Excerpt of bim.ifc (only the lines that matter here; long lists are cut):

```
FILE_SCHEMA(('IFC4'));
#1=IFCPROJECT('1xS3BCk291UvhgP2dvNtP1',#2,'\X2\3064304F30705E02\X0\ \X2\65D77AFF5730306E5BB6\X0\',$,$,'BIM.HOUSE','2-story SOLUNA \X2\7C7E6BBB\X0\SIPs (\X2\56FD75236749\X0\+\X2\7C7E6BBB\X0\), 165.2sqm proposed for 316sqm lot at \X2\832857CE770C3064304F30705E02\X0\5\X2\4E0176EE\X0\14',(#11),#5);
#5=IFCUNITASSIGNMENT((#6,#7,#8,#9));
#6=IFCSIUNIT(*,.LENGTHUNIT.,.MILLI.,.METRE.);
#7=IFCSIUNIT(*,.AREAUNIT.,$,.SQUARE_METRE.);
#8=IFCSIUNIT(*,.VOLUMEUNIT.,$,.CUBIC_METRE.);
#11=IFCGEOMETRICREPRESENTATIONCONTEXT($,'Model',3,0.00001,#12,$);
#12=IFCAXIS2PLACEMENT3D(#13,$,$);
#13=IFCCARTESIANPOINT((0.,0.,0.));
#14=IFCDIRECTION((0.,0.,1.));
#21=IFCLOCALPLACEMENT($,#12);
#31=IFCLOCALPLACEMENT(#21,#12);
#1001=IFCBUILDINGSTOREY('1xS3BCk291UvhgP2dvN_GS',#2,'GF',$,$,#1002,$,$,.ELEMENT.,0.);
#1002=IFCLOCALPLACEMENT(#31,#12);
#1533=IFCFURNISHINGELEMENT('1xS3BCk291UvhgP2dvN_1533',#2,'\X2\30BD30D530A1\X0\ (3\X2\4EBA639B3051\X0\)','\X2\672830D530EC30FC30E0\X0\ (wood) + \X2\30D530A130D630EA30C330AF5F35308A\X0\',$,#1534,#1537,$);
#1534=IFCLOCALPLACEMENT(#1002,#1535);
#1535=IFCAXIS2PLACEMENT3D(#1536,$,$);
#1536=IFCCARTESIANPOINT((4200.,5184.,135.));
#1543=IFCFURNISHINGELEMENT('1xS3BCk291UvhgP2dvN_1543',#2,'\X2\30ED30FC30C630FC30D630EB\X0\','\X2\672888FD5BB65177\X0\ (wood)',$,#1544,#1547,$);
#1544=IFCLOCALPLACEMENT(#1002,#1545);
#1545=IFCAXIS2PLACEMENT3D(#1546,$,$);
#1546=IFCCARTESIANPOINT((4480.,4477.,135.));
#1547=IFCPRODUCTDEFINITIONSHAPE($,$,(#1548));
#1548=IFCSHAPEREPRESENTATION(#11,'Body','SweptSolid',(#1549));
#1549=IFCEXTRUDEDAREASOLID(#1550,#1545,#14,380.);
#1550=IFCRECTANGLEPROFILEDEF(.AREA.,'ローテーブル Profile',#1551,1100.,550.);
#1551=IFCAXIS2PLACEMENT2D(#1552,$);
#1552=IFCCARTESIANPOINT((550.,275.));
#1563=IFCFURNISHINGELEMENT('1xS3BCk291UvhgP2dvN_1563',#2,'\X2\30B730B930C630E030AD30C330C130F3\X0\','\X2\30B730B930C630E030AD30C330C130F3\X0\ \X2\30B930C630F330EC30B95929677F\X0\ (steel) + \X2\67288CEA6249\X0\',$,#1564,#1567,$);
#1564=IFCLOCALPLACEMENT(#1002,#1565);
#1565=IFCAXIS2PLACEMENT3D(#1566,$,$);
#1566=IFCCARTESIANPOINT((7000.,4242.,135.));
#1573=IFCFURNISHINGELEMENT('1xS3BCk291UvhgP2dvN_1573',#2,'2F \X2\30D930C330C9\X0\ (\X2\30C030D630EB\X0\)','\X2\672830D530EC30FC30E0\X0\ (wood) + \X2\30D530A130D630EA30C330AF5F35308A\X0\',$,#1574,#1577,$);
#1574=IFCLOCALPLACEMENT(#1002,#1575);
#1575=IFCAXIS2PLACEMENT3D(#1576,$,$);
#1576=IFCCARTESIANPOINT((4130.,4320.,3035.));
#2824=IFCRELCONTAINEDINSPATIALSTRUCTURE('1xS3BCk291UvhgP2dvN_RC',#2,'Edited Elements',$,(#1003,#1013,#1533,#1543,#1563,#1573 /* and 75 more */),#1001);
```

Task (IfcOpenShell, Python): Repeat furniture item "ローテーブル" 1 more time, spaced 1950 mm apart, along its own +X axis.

```python
import ifcopenshell
import ifcopenshell.api.geometry
import ifcopenshell.api.root
import ifcopenshell.util.element
import ifcopenshell.util.placement

model = ifcopenshell.open("bim.ifc")


def reuse_history(source, copy):
    """copy_class also copies each property set's owner history, people and application; keep the originals."""
    for rel in copy.IsDefinedBy:
        if rel.is_a("IfcRelDefinesByProperties") and (history := rel.RelatingPropertyDefinition.OwnerHistory):
            rel.RelatingPropertyDefinition.OwnerHistory = source.OwnerHistory
            ifcopenshell.util.element.remove_deep2(model, history)


source = model.by_id(1543)
base = ifcopenshell.util.placement.get_local_placement(source.ObjectPlacement)
step = base[:3, 0] * 1950.0

for i in range(1, 2):
    copy = ifcopenshell.api.root.copy_class(model, product=source)
    copy.Representation = ifcopenshell.util.element.copy_deep(
        model, source.Representation, exclude=["IfcGeometricRepresentationContext", "IfcRepresentationMap"]
    )
    reuse_history(source, copy)
    matrix = base.copy()
    matrix[:3, 3] += i * step
    print("added at", matrix[:3, 3].round(3) + 0.0)
    ifcopenshell.api.geometry.edit_object_placement(model, product=copy, matrix=matrix, is_si=False)

model.write("bim_v2.ifc")
```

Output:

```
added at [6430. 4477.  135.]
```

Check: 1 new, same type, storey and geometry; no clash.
